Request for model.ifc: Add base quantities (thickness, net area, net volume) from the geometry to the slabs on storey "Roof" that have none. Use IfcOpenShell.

First a look at what the model holds.

```python
import ifcopenshell
import ifcopenshell.util.element
import ifcopenshell.util.unit

model = ifcopenshell.open("model.ifc")
print(model.schema)
for unit_type in ("LENGTHUNIT", "AREAUNIT", "VOLUMEUNIT"):
    print(unit_type, ifcopenshell.util.unit.calculate_unit_scale(model, unit_type))
storey = next(s for s in model.by_type("IfcBuildingStorey") if s.Name == "Roof")
slabs = [e for e in ifcopenshell.util.element.get_decomposition(storey) if e.is_a("IfcSlab")]
for e in sorted(slabs, key=lambda e: e.id()):
    print(e.id(), e.is_a(), e.Name, list(ifcopenshell.util.element.get_psets(e, qtos_only=True)), sep=" | ")
```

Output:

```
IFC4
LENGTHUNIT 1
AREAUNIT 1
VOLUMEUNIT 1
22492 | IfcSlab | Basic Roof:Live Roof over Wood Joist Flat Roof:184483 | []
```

```python
import ifcopenshell
import ifcopenshell.api.pset
import ifcopenshell.geom
import ifcopenshell.util.element
import ifcopenshell.util.shape
import ifcopenshell.util.unit

model = ifcopenshell.open("model.ifc")
unit_scale = ifcopenshell.util.unit.calculate_unit_scale(model)
area_scale = ifcopenshell.util.unit.calculate_unit_scale(model, "AREAUNIT")
volume_scale = ifcopenshell.util.unit.calculate_unit_scale(model, "VOLUMEUNIT")
settings = ifcopenshell.geom.settings()

storey = next(s for s in model.by_type("IfcBuildingStorey") if s.Name == "Roof")
slabs = [e for e in ifcopenshell.util.element.get_decomposition(storey) if e.is_a("IfcSlab")]

for e in sorted(slabs, key=lambda e: e.id()):
    if ifcopenshell.util.element.get_psets(e, qtos_only=True, should_inherit=False):
        continue
    # Geometry comes back in metres, in the element's own axes.
    shape = ifcopenshell.geom.create_shape(settings, e)
    values = {
        "Width": ifcopenshell.util.shape.get_z(shape.geometry) / unit_scale,
        "NetArea": ifcopenshell.util.shape.get_footprint_area(shape.geometry) / area_scale,
        "NetVolume": ifcopenshell.util.shape.get_volume(shape.geometry) / volume_scale,
    }
    qto = ifcopenshell.api.pset.add_qto(model, product=e, name="Qto_SlabBaseQuantities")
    ifcopenshell.api.pset.edit_qto(model, qto=qto, properties=values)
    print(e.id(), {k: round(v, 3) for k, v in values.items()})

model.write("model_edited.ifc")
```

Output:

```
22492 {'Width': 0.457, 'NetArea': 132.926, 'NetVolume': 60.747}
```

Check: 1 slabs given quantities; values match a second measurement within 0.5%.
